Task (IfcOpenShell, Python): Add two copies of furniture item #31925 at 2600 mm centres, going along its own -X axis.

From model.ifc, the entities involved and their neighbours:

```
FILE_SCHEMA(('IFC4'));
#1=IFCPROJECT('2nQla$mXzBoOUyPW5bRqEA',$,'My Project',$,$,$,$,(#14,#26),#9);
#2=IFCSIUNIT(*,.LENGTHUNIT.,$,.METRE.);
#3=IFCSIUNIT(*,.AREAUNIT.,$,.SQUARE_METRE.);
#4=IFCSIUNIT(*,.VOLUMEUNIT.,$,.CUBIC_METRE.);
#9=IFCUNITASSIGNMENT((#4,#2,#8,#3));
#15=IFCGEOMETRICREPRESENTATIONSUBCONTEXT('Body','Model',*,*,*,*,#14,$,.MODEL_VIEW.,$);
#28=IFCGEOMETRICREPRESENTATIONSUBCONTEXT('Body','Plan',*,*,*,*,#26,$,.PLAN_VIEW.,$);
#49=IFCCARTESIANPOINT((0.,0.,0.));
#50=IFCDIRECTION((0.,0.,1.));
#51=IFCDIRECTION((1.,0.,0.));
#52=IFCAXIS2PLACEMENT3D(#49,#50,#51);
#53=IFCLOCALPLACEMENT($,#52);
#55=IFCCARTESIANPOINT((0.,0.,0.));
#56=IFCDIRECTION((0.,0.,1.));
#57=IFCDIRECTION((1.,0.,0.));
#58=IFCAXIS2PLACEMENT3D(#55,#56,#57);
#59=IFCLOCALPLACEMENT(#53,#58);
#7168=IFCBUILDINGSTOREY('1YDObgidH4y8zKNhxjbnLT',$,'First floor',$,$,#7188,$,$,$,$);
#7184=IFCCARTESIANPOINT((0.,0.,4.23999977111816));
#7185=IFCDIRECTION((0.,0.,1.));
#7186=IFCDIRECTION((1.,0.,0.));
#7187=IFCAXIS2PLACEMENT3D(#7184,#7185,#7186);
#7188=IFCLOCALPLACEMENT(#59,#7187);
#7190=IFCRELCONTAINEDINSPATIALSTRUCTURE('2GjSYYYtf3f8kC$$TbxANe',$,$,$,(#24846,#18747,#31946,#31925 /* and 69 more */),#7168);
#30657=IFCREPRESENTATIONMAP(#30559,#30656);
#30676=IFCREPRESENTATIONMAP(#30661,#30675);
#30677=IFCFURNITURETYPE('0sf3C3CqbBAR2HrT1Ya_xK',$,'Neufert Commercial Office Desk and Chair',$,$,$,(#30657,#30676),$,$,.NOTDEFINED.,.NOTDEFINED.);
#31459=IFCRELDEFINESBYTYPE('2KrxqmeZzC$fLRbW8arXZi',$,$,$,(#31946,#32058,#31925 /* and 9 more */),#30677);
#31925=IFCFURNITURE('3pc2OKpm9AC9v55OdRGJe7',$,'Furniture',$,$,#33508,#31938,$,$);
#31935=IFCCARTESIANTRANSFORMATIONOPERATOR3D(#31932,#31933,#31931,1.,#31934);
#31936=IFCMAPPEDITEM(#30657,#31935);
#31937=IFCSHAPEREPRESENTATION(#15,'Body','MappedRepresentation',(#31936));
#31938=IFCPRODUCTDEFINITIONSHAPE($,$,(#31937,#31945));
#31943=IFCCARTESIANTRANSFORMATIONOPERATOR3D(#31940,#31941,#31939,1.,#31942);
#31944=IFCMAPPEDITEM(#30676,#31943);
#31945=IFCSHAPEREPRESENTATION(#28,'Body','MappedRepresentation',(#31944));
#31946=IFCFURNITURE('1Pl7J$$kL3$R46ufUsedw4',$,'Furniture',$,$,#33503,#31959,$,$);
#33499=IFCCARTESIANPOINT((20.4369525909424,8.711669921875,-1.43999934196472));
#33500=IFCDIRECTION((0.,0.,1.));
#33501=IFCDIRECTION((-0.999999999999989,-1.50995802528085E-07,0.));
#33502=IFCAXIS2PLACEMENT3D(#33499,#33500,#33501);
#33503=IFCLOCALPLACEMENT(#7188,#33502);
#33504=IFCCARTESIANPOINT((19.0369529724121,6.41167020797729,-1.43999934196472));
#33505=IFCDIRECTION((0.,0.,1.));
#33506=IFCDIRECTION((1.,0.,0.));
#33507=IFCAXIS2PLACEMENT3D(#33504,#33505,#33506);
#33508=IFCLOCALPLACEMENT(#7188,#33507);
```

```python
import ifcopenshell
import ifcopenshell.api.geometry
import ifcopenshell.api.root
import ifcopenshell.util.element
import ifcopenshell.util.placement
import ifcopenshell.util.unit

model = ifcopenshell.open("model.ifc")
unit_scale = ifcopenshell.util.unit.calculate_unit_scale(model)

source = model.by_guid("3pc2OKpm9AC9v55OdRGJe7")
base = ifcopenshell.util.placement.get_local_placement(source.ObjectPlacement)
step = -base[:3, 0] * 2.6 / unit_scale

for i in range(1, 3):
    copy = ifcopenshell.api.root.copy_class(model, product=source)
    copy.Representation = ifcopenshell.util.element.copy_deep(
        model, source.Representation, exclude=["IfcGeometricRepresentationContext", "IfcRepresentationMap"]
    )
    matrix = base.copy()
    matrix[:3, 3] += i * step
    print("added at", matrix[:3, 3].round(3) + 0.0)
    ifcopenshell.api.geometry.edit_object_placement(model, product=copy, matrix=matrix, is_si=False)

model.write("model_edited.ifc")
```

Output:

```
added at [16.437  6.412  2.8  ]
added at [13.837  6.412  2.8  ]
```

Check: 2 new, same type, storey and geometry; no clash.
